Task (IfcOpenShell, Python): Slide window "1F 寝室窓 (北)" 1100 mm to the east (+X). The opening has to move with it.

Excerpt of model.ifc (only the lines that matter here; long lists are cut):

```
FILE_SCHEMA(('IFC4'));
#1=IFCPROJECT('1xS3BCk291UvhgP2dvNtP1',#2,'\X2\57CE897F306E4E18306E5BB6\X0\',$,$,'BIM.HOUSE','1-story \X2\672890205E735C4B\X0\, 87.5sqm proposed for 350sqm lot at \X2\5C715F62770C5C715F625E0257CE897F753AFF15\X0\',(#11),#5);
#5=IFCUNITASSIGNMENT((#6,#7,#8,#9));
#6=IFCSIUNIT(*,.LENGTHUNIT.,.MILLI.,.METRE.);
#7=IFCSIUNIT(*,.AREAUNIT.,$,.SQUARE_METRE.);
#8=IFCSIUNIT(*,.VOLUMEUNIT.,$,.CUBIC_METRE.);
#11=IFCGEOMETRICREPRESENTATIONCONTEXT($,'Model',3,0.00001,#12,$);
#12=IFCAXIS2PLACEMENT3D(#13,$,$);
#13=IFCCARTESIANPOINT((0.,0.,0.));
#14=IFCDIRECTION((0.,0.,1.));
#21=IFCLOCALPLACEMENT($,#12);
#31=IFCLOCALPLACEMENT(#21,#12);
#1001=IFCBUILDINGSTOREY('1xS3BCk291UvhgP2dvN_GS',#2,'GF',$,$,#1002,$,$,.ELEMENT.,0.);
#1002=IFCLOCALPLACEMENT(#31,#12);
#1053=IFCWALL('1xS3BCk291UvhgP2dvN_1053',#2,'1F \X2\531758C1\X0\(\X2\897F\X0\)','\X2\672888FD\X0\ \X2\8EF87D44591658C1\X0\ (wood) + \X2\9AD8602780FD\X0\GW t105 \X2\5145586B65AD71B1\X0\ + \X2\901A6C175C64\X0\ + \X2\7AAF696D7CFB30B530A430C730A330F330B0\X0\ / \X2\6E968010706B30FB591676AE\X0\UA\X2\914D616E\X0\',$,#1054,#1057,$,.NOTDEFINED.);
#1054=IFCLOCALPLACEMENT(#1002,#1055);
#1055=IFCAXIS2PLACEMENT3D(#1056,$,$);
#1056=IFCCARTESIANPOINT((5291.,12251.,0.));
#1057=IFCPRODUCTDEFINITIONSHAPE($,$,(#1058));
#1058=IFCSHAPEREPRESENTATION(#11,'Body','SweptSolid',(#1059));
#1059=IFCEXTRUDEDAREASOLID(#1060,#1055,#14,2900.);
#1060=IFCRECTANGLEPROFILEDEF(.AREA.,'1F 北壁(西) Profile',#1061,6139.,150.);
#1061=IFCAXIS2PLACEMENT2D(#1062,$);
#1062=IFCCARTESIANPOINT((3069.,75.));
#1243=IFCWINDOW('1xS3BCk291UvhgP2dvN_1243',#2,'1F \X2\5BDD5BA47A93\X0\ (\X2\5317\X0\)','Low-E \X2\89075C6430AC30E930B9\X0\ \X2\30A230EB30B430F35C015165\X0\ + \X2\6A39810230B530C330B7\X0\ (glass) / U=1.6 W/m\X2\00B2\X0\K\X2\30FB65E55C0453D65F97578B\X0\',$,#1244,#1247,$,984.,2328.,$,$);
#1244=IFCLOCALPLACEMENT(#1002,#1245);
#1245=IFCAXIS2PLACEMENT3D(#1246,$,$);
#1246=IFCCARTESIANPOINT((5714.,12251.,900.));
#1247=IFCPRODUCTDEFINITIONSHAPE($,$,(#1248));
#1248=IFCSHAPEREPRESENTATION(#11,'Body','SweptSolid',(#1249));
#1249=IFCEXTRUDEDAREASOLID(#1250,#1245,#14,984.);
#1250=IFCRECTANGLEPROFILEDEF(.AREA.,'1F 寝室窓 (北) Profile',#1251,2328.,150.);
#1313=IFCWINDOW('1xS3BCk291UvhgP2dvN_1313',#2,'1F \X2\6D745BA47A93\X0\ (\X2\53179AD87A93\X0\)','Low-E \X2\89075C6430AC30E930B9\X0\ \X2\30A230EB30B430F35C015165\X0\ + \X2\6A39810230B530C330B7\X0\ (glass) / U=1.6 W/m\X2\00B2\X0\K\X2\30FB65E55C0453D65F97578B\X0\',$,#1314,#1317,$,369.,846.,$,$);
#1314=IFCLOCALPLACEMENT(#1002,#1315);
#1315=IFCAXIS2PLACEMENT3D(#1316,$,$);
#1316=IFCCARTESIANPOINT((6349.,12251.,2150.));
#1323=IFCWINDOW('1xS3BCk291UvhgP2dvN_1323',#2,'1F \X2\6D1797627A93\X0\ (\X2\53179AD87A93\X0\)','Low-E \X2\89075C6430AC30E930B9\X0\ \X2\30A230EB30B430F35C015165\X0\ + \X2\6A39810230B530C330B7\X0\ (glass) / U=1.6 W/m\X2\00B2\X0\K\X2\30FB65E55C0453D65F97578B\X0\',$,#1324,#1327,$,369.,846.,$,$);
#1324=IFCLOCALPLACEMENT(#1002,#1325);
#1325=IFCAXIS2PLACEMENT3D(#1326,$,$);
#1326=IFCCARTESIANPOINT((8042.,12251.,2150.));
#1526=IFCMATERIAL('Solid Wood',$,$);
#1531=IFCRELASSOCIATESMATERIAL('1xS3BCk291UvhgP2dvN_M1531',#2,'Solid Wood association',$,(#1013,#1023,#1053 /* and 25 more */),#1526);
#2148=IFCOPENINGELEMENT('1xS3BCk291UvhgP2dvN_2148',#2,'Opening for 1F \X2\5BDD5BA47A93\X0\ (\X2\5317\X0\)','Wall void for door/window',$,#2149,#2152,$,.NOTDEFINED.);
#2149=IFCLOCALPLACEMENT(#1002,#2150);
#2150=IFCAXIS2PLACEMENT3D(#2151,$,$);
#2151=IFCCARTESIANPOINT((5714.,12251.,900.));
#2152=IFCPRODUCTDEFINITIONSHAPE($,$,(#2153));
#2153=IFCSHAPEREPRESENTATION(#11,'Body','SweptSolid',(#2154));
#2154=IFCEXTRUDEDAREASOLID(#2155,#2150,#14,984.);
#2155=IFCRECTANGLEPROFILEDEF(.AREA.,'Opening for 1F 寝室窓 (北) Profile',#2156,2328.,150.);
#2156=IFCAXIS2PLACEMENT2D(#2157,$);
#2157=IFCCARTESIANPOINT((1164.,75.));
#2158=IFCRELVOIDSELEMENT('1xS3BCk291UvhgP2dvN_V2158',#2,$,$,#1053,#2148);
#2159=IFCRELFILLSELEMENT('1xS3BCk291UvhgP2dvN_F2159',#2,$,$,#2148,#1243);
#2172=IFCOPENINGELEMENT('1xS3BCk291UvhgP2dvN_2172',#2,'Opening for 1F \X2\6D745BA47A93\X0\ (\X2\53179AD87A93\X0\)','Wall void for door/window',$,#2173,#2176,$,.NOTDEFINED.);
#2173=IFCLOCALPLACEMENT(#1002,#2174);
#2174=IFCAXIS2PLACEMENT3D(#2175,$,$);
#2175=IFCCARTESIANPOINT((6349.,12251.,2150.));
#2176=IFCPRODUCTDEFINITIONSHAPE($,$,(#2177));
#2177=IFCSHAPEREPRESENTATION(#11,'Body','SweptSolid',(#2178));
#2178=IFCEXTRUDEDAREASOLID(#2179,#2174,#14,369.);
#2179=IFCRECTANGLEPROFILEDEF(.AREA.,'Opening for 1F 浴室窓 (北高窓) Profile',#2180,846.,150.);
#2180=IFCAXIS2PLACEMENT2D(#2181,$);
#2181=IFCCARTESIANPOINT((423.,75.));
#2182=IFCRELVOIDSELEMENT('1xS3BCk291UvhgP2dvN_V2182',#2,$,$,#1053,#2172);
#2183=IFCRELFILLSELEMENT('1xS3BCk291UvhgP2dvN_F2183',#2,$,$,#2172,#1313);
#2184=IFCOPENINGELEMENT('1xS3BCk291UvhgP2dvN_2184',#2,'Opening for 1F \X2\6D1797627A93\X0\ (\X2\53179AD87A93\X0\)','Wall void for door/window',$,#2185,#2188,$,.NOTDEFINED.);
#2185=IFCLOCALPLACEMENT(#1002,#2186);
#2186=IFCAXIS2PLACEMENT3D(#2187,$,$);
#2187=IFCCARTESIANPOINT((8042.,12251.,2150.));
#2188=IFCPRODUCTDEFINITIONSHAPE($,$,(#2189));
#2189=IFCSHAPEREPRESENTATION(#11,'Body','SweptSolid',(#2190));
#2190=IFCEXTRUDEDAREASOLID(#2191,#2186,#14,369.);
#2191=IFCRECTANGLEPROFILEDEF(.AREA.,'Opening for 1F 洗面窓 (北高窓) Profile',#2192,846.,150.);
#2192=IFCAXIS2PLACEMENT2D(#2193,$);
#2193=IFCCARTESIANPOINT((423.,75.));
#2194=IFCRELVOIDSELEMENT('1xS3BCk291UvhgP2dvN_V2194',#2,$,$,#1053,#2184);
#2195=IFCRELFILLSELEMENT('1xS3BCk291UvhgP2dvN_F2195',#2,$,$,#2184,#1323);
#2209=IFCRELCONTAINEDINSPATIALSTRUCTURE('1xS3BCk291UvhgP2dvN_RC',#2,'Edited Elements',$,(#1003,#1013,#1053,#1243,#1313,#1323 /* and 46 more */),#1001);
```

```python
import ifcopenshell
import ifcopenshell.api.geometry
import ifcopenshell.util.placement
import ifcopenshell.util.unit

model = ifcopenshell.open("model.ifc")
unit_scale = ifcopenshell.util.unit.calculate_unit_scale(model)

window = model.by_id(1243)
opening = window.FillsVoids[0].RelatingOpeningElement
wall = opening.VoidsElements[0].RelatingBuildingElement

wall_matrix = ifcopenshell.util.placement.get_local_placement(wall.ObjectPlacement)
shift = wall_matrix[:3, 0] * 1.1 / unit_scale
before = ifcopenshell.util.placement.get_local_placement(window.ObjectPlacement)[:3, 3].copy()

# The window is not placed relative to its opening, so move both.
for product in (opening, window):
    matrix = ifcopenshell.util.placement.get_local_placement(product.ObjectPlacement)
    matrix[:3, 3] += shift
    ifcopenshell.api.geometry.edit_object_placement(model, product=product, matrix=matrix, is_si=False)

after = ifcopenshell.util.placement.get_local_placement(window.ObjectPlacement)[:3, 3]
print("window moved by", (after - before).round(3) + 0.0)

model.write("model-out.ifc")
```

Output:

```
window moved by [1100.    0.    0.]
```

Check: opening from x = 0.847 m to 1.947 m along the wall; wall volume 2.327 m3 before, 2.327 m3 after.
